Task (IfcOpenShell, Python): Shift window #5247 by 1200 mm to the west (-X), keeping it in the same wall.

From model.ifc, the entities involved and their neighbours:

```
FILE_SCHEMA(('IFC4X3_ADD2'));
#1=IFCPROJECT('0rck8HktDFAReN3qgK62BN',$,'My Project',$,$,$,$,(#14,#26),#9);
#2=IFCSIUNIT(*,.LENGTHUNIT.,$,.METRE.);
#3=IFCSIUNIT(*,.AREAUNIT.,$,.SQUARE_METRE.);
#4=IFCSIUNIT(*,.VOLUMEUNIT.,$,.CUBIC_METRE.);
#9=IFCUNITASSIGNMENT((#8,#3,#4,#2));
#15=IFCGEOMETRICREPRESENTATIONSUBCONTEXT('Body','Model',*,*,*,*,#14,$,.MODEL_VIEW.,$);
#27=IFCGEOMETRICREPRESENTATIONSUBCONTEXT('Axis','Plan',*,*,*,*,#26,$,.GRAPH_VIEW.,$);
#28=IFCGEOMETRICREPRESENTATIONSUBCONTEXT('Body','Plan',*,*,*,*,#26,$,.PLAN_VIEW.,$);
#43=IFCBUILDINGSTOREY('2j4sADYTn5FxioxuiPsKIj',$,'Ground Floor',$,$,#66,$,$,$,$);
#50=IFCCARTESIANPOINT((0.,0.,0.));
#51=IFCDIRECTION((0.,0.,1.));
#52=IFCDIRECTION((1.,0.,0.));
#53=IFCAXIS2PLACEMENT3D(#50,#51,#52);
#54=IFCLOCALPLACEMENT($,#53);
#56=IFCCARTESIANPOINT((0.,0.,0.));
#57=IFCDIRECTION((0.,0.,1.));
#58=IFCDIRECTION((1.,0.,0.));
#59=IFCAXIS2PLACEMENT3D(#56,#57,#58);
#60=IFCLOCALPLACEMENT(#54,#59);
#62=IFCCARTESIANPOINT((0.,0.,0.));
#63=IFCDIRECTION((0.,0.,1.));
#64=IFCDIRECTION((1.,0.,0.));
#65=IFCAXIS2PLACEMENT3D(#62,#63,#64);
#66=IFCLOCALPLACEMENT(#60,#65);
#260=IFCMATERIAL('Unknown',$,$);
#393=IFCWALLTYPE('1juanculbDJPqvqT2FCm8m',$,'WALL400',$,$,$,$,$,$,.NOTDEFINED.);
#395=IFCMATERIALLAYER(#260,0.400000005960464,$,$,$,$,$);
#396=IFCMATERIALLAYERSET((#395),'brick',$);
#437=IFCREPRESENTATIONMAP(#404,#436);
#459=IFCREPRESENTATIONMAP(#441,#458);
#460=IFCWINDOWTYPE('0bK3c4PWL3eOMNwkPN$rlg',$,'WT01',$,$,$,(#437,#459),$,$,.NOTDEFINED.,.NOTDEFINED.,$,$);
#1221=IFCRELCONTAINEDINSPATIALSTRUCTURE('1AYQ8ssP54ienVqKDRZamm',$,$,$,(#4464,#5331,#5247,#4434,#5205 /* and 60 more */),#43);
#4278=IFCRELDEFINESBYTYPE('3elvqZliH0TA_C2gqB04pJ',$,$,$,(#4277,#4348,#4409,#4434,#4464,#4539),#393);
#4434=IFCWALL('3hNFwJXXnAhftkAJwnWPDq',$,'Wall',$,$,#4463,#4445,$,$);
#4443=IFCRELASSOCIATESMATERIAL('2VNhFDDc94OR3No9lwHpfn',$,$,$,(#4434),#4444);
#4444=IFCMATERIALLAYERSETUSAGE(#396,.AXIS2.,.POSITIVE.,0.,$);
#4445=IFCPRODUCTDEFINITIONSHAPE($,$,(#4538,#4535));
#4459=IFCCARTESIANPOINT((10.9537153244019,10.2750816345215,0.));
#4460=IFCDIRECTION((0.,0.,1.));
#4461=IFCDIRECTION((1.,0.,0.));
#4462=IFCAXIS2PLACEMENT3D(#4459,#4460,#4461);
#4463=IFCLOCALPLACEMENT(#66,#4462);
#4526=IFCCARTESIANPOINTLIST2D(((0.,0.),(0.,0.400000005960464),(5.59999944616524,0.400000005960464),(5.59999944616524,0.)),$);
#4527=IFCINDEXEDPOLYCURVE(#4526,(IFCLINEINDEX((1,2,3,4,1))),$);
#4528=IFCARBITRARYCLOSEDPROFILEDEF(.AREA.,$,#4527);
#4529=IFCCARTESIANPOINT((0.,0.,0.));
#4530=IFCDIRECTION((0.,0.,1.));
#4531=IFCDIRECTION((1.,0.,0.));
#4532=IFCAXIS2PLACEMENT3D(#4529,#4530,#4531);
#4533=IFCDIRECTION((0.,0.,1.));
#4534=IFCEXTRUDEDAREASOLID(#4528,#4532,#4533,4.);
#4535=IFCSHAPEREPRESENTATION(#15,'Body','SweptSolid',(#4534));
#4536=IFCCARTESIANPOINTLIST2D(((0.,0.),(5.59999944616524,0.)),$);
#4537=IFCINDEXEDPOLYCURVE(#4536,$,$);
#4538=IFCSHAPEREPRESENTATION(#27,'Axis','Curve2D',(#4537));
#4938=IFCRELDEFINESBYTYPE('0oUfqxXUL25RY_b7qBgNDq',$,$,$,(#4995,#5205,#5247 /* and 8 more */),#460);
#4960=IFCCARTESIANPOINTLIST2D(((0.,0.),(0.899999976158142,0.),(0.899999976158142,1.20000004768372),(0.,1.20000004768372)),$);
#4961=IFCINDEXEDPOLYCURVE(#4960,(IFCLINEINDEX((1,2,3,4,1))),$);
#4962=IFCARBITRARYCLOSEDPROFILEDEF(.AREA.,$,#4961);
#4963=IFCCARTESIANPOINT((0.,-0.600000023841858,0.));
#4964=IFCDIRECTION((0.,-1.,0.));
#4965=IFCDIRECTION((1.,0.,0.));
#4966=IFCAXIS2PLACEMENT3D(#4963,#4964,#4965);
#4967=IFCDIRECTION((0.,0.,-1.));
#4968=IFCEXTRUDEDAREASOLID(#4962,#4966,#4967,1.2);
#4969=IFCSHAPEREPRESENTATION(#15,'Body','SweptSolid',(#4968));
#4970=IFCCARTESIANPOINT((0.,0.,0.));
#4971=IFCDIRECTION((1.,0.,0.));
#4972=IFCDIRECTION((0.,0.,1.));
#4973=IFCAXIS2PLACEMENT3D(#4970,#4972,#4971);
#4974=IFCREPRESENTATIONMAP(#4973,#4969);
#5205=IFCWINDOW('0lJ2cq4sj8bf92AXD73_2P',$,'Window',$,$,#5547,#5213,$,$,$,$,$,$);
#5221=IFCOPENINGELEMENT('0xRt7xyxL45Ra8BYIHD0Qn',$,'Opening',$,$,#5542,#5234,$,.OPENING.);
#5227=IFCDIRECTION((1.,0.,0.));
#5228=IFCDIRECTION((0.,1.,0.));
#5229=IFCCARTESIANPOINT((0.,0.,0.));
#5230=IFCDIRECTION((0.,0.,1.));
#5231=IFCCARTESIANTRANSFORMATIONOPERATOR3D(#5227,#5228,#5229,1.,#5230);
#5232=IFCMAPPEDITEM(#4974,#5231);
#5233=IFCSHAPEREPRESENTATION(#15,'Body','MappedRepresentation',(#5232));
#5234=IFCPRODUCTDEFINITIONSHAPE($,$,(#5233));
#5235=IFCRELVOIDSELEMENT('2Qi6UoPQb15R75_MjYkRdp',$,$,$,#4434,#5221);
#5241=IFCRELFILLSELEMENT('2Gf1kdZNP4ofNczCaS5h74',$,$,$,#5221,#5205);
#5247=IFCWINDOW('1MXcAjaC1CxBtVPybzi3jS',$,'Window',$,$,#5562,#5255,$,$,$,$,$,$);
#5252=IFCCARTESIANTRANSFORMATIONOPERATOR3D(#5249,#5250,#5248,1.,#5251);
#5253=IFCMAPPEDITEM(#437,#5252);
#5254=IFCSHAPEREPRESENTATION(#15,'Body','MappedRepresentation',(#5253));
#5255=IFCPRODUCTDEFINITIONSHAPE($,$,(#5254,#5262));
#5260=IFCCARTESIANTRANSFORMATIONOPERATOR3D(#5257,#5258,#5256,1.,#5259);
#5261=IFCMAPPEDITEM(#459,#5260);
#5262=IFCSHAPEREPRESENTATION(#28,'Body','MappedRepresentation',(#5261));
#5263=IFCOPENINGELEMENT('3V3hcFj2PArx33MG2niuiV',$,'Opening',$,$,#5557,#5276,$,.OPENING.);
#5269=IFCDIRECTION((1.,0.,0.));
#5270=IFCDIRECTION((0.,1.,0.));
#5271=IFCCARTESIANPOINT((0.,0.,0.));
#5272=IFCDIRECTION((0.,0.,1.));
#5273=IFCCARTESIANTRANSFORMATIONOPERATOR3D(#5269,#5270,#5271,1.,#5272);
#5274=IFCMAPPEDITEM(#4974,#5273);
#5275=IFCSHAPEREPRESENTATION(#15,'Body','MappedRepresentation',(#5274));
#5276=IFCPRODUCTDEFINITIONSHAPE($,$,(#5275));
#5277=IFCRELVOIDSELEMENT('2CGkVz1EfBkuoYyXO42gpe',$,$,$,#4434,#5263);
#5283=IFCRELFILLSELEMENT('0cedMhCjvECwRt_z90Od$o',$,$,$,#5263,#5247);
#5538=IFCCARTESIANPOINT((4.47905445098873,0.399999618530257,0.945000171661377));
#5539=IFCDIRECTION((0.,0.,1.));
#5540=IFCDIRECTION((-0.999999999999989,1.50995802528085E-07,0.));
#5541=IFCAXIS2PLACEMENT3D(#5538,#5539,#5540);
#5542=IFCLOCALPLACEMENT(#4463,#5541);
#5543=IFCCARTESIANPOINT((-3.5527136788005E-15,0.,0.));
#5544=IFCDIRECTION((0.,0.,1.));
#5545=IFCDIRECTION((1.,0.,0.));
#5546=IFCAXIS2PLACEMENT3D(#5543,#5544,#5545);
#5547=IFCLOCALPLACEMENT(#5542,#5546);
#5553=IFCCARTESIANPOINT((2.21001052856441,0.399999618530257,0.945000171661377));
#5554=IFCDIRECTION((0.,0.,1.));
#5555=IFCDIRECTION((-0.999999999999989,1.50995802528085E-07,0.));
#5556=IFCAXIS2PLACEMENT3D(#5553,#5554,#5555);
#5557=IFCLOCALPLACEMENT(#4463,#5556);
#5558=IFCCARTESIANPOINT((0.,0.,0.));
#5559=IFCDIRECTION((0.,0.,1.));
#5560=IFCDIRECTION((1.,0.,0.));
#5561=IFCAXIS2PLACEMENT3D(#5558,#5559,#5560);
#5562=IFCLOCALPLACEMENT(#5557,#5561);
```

```python
import ifcopenshell
import ifcopenshell.api.geometry
import ifcopenshell.util.placement
import ifcopenshell.util.unit

model = ifcopenshell.open("model.ifc")
unit_scale = ifcopenshell.util.unit.calculate_unit_scale(model)

window = model.by_guid("1MXcAjaC1CxBtVPybzi3jS")
opening = window.FillsVoids[0].RelatingOpeningElement
wall = opening.VoidsElements[0].RelatingBuildingElement

wall_matrix = ifcopenshell.util.placement.get_local_placement(wall.ObjectPlacement)
shift = wall_matrix[:3, 0] * -1.2 / unit_scale
before = ifcopenshell.util.placement.get_local_placement(window.ObjectPlacement)[:3, 3].copy()

# The window is placed relative to its opening, so it follows when the opening moves.
matrix = ifcopenshell.util.placement.get_local_placement(opening.ObjectPlacement)
matrix[:3, 3] += shift
ifcopenshell.api.geometry.edit_object_placement(
    model, product=opening, matrix=matrix, is_si=False, should_transform_children=True
)

after = ifcopenshell.util.placement.get_local_placement(window.ObjectPlacement)[:3, 3]
print("window moved by", (after - before).round(3) + 0.0)

model.write("model-out.ifc")
```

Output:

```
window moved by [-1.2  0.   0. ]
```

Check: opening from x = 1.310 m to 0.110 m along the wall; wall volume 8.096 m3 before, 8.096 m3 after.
